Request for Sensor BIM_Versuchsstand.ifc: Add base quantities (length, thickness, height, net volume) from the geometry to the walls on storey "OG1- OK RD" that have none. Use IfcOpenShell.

First a look at what the model holds.

```python
import ifcopenshell
import ifcopenshell.util.element
import ifcopenshell.util.unit

model = ifcopenshell.open("Sensor BIM_Versuchsstand.ifc")
print(model.schema)
for unit_type in ("LENGTHUNIT", "AREAUNIT", "VOLUMEUNIT"):
    print(unit_type, ifcopenshell.util.unit.calculate_unit_scale(model, unit_type))
storey = next(s for s in model.by_type("IfcBuildingStorey") if s.Name == "OG1- OK RD")
walls = [e for e in ifcopenshell.util.element.get_decomposition(storey) if e.is_a("IfcWall")]
for e in sorted(walls, key=lambda e: e.id()):
    print(e.id(), e.is_a(), e.Name, list(ifcopenshell.util.element.get_psets(e, qtos_only=True)), sep=" | ")
```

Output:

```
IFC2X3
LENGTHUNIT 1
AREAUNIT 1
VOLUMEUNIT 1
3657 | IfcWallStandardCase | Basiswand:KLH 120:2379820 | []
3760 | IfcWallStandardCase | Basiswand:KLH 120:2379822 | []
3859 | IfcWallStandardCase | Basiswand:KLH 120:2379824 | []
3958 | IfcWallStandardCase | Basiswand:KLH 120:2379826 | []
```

```python
import ifcopenshell
import ifcopenshell.api.pset
import ifcopenshell.geom
import ifcopenshell.util.element
import ifcopenshell.util.shape
import ifcopenshell.util.unit

model = ifcopenshell.open("Sensor BIM_Versuchsstand.ifc")
unit_scale = ifcopenshell.util.unit.calculate_unit_scale(model)
volume_scale = ifcopenshell.util.unit.calculate_unit_scale(model, "VOLUMEUNIT")
settings = ifcopenshell.geom.settings()

storey = next(s for s in model.by_type("IfcBuildingStorey") if s.Name == "OG1- OK RD")
walls = [e for e in ifcopenshell.util.element.get_decomposition(storey) if e.is_a("IfcWall")]

for e in sorted(walls, key=lambda e: e.id()):
    if ifcopenshell.util.element.get_psets(e, qtos_only=True, should_inherit=False):
        continue
    # Geometry comes back in metres, in the element's own axes.
    shape = ifcopenshell.geom.create_shape(settings, e)
    values = {
        "Length": ifcopenshell.util.shape.get_x(shape.geometry) / unit_scale,
        "Width": ifcopenshell.util.shape.get_y(shape.geometry) / unit_scale,
        "Height": ifcopenshell.util.shape.get_z(shape.geometry) / unit_scale,
        "NetVolume": ifcopenshell.util.shape.get_volume(shape.geometry) / volume_scale,
    }
    qto = ifcopenshell.api.pset.add_qto(model, product=e, name="BaseQuantities")
    ifcopenshell.api.pset.edit_qto(model, qto=qto, properties=values)
    print(e.id(), {k: round(v, 3) for k, v in values.items()})

model.write("Sensor BIM_Versuchsstand-out.ifc")
```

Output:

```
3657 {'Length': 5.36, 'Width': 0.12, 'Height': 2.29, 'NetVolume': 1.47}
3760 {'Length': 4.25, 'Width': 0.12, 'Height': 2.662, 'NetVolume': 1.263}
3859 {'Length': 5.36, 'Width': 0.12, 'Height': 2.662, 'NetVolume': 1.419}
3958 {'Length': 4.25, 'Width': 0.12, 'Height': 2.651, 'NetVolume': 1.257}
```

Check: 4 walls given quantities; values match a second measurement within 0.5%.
